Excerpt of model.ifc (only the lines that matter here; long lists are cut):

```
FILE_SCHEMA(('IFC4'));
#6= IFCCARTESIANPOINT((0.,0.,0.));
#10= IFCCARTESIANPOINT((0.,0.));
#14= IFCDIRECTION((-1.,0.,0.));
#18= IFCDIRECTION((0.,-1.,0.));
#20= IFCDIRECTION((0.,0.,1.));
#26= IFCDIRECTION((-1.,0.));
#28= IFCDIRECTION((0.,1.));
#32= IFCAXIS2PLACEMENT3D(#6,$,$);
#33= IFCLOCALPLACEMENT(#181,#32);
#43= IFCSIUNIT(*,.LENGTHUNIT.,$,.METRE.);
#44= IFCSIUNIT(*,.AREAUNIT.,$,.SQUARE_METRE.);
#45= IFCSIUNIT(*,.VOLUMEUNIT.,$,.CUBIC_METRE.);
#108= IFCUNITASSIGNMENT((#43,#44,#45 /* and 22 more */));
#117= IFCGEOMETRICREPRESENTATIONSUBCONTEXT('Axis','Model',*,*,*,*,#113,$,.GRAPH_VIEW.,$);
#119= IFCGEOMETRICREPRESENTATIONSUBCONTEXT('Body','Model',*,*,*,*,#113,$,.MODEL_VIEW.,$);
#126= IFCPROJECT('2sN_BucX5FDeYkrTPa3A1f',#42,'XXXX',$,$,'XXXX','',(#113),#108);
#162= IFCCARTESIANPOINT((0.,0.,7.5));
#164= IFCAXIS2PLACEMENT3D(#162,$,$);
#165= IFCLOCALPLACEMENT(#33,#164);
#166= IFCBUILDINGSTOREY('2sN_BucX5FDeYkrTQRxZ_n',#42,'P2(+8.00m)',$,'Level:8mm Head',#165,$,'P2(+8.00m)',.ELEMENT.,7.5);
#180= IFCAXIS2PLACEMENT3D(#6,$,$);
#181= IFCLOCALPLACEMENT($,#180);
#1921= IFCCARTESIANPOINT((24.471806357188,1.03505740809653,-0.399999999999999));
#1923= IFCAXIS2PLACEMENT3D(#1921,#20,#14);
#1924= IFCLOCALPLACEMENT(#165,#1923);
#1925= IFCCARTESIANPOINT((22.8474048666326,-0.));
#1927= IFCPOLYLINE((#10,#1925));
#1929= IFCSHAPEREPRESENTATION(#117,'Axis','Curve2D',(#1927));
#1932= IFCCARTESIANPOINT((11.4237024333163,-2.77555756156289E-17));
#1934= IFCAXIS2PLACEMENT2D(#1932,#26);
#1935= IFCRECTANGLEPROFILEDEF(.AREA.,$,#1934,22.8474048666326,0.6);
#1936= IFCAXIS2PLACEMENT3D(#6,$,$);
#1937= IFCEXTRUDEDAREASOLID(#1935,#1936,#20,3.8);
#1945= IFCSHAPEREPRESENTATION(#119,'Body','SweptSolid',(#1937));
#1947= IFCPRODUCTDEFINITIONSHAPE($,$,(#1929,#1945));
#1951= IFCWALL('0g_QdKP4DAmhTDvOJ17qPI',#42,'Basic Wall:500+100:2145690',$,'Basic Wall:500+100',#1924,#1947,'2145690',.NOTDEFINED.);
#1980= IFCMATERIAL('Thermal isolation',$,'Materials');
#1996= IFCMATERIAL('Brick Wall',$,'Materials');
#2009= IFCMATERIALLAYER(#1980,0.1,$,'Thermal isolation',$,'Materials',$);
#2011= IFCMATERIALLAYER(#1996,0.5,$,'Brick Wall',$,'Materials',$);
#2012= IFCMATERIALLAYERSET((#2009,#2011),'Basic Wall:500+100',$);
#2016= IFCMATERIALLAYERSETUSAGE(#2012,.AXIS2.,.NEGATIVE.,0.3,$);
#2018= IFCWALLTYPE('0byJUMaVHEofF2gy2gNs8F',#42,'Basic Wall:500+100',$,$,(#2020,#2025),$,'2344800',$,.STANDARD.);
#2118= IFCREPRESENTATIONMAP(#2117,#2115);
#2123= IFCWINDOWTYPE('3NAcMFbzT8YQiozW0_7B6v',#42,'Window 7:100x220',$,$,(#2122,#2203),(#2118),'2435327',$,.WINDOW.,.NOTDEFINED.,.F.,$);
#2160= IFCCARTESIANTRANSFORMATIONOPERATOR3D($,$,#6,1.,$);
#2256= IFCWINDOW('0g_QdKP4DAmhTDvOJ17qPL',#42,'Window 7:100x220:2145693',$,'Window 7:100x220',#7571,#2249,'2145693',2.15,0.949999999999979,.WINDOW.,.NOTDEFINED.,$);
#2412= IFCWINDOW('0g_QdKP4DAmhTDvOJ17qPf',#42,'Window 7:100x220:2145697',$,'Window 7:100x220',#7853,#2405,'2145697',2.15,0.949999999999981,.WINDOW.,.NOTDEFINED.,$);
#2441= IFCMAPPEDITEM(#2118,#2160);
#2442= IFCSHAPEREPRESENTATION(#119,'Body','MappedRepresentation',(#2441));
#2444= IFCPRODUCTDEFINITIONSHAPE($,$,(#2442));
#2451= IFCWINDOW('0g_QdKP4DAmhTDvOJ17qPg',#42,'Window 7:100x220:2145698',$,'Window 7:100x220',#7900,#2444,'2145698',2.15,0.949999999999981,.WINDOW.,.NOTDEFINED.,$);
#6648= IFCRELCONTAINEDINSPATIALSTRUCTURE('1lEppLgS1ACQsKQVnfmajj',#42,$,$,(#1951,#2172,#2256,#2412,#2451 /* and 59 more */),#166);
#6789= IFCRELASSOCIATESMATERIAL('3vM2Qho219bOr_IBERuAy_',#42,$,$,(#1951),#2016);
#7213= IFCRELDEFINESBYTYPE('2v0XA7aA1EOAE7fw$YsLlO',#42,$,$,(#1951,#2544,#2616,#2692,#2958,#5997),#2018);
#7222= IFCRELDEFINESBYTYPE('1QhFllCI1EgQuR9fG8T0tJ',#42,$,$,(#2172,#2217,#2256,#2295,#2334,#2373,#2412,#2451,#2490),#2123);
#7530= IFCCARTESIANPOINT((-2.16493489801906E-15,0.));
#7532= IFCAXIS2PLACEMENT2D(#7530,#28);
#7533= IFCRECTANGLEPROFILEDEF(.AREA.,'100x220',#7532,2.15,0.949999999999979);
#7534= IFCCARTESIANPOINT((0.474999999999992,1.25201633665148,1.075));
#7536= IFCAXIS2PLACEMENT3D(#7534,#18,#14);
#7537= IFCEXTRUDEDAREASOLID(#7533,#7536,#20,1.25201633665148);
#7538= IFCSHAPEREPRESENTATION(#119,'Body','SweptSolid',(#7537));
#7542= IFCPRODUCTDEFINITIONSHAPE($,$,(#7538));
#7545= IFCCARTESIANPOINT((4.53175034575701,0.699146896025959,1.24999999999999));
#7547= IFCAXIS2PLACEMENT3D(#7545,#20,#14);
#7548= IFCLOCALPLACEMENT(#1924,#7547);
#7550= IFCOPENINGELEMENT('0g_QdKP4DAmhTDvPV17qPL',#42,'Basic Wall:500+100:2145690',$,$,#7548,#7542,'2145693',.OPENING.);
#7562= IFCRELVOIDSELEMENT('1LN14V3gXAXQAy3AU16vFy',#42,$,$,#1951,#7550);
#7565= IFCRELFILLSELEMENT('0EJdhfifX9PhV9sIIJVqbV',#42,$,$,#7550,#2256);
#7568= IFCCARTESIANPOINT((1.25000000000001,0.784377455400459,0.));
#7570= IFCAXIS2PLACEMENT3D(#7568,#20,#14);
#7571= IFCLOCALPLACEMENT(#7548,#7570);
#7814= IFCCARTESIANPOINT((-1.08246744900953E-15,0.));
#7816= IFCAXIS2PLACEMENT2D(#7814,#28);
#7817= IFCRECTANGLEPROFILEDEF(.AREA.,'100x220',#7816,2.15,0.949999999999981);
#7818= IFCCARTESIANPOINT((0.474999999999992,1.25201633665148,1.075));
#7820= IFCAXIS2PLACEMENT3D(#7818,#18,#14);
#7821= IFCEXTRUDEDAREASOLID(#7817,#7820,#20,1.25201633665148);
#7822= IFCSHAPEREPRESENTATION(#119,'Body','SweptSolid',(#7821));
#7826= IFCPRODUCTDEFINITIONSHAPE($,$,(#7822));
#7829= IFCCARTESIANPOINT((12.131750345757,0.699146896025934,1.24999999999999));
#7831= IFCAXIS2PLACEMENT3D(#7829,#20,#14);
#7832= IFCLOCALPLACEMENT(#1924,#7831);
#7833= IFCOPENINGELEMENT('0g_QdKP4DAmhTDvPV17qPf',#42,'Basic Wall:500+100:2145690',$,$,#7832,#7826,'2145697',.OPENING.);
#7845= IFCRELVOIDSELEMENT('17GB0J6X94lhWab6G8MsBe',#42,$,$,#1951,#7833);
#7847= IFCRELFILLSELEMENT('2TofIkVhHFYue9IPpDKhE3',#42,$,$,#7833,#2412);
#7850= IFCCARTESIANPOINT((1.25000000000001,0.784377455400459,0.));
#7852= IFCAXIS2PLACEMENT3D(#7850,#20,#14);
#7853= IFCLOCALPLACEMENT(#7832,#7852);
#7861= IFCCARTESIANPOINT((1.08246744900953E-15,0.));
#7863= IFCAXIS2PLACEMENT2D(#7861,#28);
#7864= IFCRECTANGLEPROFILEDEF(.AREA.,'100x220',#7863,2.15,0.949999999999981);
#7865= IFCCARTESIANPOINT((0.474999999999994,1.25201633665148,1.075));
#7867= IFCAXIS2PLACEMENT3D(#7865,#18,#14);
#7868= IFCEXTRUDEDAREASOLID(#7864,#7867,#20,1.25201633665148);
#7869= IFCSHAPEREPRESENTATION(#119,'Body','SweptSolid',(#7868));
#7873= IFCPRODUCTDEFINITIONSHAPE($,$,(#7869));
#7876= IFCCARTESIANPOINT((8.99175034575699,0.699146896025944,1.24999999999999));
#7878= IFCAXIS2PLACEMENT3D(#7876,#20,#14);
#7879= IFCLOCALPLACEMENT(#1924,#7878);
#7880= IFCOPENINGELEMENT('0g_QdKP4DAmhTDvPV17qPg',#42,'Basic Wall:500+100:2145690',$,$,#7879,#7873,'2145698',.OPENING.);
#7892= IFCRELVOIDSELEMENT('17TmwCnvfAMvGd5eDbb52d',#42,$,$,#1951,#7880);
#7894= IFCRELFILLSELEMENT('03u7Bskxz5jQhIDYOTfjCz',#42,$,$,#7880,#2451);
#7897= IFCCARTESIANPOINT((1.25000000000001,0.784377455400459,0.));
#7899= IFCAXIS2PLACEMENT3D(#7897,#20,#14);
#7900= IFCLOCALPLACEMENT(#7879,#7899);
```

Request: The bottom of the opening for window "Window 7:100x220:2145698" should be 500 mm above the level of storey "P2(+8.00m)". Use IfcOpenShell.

```python
import numpy as np
import ifcopenshell
import ifcopenshell.api.geometry
import ifcopenshell.geom
import ifcopenshell.util.element
import ifcopenshell.util.placement
import ifcopenshell.util.shape
import ifcopenshell.util.unit

model = ifcopenshell.open("model.ifc")
unit_scale = ifcopenshell.util.unit.calculate_unit_scale(model)

window = model.by_guid("0g_QdKP4DAmhTDvOJ17qPg")
opening = window.FillsVoids[0].RelatingOpeningElement
storey = ifcopenshell.util.element.get_container(window, ifc_class="IfcBuildingStorey")
level = ifcopenshell.util.placement.get_local_placement(storey.ObjectPlacement)[2, 3]

# The opening's origin need not be at the sill, so measure its lowest point.
shape = ifcopenshell.geom.create_shape(ifcopenshell.geom.settings(), opening)
bottom = ifcopenshell.util.shape.get_shape_bottom_elevation(shape, shape.geometry) / unit_scale
dz = level + 0.5 / unit_scale - bottom

shift = np.array([0.0, 0.0, dz])
# The window is placed relative to its opening, so it follows when the opening moves.
matrix = ifcopenshell.util.placement.get_local_placement(opening.ObjectPlacement)
matrix[:3, 3] += shift
ifcopenshell.api.geometry.edit_object_placement(
    model, product=opening, matrix=matrix, is_si=False, should_transform_children=True
)

print(f"moved by {dz * unit_scale:+.3f} m")

model.write("model-out.ifc")
```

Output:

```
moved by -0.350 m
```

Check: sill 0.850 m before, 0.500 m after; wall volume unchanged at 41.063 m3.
